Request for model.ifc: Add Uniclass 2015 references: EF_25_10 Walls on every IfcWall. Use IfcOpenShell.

First a look at what the model holds.

```python
import ifcopenshell

model = ifcopenshell.open("model.ifc")
print(model.schema)
print("classifications:", [c.Name for c in model.by_type("IfcClassification")])
for ifc_class in ("IfcDoor", "IfcRoof", "IfcStair", "IfcWall", "IfcWindow"):
    print(ifc_class, len(model.by_type(ifc_class)))
```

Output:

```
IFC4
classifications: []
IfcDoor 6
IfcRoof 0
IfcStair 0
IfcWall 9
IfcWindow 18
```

```python
import ifcopenshell
import ifcopenshell.api.classification

model = ifcopenshell.open("model.ifc")

system = ifcopenshell.api.classification.add_classification(model, classification="Uniclass 2015")

codes = {
    "IfcWall": ("EF_25_10", "Walls"),
}
for ifc_class, (code, name) in codes.items():
    products = model.by_type(ifc_class)
    ifcopenshell.api.classification.add_reference(
        model, products=products, classification=system, identification=code, name=name
    )
    print(code, len(products))

model.write("model_updated.ifc")
```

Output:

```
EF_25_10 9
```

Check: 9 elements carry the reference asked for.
